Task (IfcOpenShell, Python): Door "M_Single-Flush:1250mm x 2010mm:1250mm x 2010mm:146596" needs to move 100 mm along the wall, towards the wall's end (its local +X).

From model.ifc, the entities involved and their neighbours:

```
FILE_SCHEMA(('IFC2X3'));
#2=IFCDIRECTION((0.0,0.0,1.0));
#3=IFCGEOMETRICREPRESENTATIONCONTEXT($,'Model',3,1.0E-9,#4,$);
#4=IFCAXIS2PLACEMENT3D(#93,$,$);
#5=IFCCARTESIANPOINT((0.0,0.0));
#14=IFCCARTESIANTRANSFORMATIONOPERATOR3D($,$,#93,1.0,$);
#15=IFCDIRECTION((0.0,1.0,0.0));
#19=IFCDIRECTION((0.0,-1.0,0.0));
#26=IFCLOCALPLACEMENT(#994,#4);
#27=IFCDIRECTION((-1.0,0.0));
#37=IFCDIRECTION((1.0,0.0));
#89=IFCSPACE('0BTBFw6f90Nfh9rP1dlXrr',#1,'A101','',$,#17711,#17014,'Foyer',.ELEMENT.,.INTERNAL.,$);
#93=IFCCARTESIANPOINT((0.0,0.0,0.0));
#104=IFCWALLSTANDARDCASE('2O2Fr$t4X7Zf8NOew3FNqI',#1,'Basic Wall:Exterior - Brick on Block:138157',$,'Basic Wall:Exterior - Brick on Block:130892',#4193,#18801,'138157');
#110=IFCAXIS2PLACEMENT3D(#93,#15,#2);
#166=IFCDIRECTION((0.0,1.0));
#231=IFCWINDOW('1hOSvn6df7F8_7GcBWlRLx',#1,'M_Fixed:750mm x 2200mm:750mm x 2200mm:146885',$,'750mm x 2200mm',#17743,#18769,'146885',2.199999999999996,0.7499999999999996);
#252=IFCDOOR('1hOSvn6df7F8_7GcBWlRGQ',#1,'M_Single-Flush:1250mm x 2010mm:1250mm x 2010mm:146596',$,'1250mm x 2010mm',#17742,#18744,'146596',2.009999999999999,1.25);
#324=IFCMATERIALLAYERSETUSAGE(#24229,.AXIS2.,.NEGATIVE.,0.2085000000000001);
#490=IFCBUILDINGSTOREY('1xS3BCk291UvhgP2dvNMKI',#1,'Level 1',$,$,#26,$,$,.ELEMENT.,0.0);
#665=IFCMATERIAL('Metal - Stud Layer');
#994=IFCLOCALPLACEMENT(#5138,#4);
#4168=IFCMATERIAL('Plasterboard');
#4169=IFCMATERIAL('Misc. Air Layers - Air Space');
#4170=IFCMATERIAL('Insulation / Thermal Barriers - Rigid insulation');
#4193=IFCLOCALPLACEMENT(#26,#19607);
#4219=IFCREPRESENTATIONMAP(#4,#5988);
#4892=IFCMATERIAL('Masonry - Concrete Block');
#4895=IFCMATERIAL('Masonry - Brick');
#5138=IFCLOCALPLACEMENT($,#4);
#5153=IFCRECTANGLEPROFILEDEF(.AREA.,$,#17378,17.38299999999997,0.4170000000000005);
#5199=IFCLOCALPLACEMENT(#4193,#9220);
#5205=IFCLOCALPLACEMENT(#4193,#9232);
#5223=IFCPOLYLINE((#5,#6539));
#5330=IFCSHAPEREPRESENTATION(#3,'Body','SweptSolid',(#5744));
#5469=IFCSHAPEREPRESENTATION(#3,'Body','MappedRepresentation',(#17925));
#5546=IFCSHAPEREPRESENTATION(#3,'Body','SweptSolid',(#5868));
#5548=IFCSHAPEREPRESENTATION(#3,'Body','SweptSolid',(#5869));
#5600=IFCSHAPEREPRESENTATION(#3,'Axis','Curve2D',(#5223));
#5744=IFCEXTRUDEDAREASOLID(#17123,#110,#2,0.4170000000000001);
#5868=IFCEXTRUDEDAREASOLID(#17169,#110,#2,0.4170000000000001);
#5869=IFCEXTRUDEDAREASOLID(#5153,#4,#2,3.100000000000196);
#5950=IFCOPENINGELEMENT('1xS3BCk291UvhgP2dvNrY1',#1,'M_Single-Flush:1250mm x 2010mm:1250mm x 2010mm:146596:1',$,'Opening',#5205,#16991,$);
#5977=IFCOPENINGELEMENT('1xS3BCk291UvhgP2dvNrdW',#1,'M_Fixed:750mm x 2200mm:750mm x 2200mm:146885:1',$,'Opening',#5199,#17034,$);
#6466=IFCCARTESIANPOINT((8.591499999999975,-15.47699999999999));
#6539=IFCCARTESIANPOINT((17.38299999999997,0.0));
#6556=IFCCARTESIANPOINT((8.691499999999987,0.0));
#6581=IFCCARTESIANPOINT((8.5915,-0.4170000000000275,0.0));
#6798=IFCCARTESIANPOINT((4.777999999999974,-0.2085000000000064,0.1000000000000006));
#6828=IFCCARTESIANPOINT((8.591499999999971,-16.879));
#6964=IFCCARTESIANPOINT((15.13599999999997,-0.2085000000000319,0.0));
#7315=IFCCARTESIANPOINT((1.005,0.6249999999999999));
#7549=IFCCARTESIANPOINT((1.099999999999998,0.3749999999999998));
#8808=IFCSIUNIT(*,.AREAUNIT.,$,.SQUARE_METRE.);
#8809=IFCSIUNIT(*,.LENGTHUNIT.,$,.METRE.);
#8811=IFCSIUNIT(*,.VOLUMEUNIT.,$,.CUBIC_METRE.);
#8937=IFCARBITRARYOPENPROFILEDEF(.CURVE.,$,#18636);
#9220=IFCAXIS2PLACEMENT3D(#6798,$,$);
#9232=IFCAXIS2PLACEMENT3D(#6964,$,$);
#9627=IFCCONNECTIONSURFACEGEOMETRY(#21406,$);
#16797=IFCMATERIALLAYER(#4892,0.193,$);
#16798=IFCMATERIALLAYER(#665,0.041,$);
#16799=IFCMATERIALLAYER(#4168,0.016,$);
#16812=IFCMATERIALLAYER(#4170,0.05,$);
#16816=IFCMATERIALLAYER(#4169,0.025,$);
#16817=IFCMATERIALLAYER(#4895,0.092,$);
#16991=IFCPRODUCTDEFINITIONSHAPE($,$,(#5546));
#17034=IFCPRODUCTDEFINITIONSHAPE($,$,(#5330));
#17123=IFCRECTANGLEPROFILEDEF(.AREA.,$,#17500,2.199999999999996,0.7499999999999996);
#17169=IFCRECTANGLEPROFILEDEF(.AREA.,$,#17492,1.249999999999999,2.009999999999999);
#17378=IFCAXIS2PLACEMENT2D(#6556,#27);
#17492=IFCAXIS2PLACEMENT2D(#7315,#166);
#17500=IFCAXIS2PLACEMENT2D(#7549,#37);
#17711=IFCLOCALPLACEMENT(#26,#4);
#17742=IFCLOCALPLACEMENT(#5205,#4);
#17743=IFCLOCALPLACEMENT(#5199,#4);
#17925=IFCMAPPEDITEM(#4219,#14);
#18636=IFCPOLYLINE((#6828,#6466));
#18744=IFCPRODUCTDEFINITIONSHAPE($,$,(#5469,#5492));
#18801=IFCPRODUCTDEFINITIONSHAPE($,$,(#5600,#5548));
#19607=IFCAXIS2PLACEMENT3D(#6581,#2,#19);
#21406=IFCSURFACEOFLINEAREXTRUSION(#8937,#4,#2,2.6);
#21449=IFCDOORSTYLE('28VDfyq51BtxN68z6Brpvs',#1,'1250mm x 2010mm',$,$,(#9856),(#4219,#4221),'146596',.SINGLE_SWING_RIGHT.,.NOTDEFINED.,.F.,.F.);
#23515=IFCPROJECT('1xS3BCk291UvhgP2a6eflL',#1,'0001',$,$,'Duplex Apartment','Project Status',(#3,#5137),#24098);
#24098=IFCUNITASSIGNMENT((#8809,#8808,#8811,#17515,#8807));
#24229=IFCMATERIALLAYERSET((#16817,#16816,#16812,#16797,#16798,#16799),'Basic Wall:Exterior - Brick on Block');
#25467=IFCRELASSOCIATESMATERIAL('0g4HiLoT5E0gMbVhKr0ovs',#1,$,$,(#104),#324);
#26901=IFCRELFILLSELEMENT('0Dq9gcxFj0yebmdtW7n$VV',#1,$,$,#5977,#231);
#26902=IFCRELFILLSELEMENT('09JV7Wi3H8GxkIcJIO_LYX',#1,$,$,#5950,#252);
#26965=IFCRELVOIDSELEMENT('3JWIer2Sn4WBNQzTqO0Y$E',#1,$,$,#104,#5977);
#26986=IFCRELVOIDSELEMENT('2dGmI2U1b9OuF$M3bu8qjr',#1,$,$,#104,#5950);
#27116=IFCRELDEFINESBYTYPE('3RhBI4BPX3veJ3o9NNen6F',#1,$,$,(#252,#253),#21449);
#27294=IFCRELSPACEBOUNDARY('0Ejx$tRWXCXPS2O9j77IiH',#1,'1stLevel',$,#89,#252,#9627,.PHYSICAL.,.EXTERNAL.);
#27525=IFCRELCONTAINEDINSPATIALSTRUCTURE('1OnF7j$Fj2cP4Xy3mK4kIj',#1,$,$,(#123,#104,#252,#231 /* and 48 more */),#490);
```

```python
import numpy as np
import ifcopenshell
import ifcopenshell.api.geometry
import ifcopenshell.util.placement

model = ifcopenshell.open("model.ifc")

door = model.by_id(252)
opening = door.FillsVoids[0].RelatingOpeningElement
wall = opening.VoidsElements[0].RelatingBuildingElement

wall_matrix = ifcopenshell.util.placement.get_local_placement(wall.ObjectPlacement)
shift = wall_matrix[:3, 0] * 0.1
before = ifcopenshell.util.placement.get_local_placement(door.ObjectPlacement)[:3, 3].copy()

# The door is placed relative to its opening, so it follows when the opening moves.
matrix = ifcopenshell.util.placement.get_local_placement(opening.ObjectPlacement)
matrix[:3, 3] += shift
ifcopenshell.api.geometry.edit_object_placement(
    model, product=opening, matrix=matrix, is_si=False, should_transform_children=True
)

# Space boundary surfaces are stored in each space's coordinates; move them too.
for rel in door.ProvidesBoundaries:
    if not rel.ConnectionGeometry:
        continue
    surface = rel.ConnectionGeometry.SurfaceOnRelatingElement
    space_matrix = ifcopenshell.util.placement.get_local_placement(rel.RelatingSpace.ObjectPlacement)
    point = np.array(surface.Position.Location.Coordinates) + space_matrix[:3, :3].T @ shift
    surface.Position = model.createIfcAxis2Placement3D(
        model.createIfcCartesianPoint(point.tolist()), surface.Position.Axis, surface.Position.RefDirection
    )

after = ifcopenshell.util.placement.get_local_placement(door.ObjectPlacement)[:3, 3]
print("door moved by", (after - before).round(3) + 0.0)

model.write("model_v2.ifc")
```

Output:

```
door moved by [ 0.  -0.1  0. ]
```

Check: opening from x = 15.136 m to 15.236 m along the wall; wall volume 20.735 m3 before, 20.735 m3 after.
